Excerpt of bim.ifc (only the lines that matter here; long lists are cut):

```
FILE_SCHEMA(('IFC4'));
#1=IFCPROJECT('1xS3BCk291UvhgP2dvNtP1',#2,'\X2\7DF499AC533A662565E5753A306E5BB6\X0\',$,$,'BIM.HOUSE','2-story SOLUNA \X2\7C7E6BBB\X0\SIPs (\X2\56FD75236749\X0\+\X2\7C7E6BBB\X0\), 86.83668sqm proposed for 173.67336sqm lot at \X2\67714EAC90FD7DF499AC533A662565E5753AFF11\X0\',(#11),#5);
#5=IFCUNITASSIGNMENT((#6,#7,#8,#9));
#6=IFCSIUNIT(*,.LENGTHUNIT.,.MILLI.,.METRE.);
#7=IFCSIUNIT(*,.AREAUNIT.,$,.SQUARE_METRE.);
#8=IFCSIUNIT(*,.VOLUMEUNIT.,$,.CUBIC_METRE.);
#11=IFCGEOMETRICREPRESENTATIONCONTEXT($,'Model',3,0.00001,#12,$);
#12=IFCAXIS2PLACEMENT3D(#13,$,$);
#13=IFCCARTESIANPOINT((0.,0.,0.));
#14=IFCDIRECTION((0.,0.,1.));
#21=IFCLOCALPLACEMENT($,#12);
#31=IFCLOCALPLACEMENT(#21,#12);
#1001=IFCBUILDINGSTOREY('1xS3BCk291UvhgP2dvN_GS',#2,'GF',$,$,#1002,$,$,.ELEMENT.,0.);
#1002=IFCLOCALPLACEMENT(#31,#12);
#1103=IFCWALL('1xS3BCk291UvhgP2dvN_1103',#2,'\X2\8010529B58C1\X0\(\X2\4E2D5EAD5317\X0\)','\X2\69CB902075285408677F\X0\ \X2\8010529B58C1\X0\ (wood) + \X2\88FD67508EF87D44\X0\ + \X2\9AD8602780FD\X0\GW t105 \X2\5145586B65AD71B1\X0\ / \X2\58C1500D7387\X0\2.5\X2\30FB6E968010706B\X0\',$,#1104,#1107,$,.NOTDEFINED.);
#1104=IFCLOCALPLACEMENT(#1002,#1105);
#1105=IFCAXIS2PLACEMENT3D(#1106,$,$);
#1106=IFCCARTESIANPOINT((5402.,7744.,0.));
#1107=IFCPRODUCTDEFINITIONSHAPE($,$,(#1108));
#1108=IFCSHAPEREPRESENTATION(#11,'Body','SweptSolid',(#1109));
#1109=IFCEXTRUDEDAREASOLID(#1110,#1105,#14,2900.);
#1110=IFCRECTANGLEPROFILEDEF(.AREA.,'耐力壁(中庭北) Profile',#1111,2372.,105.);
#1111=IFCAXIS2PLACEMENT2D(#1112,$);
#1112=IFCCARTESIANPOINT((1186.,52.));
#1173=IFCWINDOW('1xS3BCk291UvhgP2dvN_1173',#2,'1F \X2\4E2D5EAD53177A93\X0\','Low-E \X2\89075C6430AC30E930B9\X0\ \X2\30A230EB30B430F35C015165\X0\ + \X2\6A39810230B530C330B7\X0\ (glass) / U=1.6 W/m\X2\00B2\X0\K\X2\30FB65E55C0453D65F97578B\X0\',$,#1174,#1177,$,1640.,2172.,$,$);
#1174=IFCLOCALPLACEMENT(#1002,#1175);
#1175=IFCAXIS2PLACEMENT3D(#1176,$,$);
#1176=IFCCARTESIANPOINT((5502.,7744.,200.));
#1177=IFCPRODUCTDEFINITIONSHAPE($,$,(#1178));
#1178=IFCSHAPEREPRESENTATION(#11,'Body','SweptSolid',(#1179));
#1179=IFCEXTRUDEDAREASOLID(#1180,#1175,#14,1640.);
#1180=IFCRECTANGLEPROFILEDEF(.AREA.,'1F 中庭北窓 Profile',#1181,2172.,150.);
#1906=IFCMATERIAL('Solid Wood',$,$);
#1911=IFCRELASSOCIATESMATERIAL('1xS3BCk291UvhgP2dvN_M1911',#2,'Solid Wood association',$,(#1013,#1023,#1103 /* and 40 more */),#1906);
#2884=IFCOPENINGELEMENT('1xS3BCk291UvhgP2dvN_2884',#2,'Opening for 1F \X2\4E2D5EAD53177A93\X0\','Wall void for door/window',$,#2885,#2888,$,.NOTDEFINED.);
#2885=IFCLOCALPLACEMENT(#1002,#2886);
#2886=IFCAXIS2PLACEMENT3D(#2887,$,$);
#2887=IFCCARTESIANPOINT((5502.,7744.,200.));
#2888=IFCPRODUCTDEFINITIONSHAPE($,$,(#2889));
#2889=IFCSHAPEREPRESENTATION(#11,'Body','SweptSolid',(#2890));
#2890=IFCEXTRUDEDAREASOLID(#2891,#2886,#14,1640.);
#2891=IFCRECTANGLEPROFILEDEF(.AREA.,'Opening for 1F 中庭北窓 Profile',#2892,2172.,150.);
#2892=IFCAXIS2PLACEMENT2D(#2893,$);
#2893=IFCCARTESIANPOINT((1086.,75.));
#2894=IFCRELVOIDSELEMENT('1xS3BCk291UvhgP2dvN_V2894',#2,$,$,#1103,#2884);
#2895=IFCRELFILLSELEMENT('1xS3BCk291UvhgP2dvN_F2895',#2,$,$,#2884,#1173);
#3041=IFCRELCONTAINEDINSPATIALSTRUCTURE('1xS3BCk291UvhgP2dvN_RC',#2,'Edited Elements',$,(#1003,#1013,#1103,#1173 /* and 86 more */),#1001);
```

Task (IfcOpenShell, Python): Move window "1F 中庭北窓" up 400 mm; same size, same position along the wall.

```python
import numpy as np
import ifcopenshell
import ifcopenshell.api.geometry
import ifcopenshell.util.placement
import ifcopenshell.util.unit

model = ifcopenshell.open("bim.ifc")
unit_scale = ifcopenshell.util.unit.calculate_unit_scale(model)

window = model.by_guid("1xS3BCk291UvhgP2dvN_1173")
opening = window.FillsVoids[0].RelatingOpeningElement
dz = 0.4 / unit_scale

shift = np.array([0.0, 0.0, dz])
# The window is not placed relative to its opening, so move both.
for product in (opening, window):
    matrix = ifcopenshell.util.placement.get_local_placement(product.ObjectPlacement)
    matrix[:3, 3] += shift
    ifcopenshell.api.geometry.edit_object_placement(model, product=product, matrix=matrix, is_si=False)

print(f"moved by {dz * unit_scale:+.3f} m")

model.write("bim_rev.ifc")
```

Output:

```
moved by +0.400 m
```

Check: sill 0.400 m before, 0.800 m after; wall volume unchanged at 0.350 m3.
